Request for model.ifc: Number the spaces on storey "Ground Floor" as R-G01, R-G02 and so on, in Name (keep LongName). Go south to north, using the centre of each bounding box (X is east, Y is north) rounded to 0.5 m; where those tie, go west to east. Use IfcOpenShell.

First a look at what the model holds.

```python
import ifcopenshell
import ifcopenshell.util.element
import ifcopenshell.util.placement

model = ifcopenshell.open("model.ifc")
print(model.schema)
storey = next(s for s in model.by_type("IfcBuildingStorey") if s.Name == "Ground Floor")
spaces = [e for e in ifcopenshell.util.element.get_decomposition(storey) if e.is_a("IfcSpace")]
for e in sorted(spaces, key=lambda e: e.id()):
    origin = ifcopenshell.util.placement.get_local_placement(e.ObjectPlacement)[:3, 3]
    print(e.id(), e.Name, e.LongName, origin.round(2) + 0.0, sep=" | ")
```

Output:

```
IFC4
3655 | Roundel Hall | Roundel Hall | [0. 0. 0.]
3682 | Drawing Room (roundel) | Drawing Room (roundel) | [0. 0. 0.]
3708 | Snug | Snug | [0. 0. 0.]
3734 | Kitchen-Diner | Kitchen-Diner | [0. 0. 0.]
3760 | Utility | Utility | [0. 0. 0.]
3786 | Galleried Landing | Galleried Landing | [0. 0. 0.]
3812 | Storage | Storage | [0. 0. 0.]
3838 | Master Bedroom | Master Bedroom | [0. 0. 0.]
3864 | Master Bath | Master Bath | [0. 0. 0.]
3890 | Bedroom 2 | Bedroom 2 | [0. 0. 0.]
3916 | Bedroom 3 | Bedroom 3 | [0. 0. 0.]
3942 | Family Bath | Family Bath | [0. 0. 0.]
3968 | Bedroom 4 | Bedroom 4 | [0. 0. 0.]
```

```python
import ifcopenshell
import ifcopenshell.geom
import ifcopenshell.util.element
import ifcopenshell.util.shape

model = ifcopenshell.open("model.ifc")
settings = ifcopenshell.geom.settings()
settings.set("use-world-coords", True)


def centre(element):
    shape = ifcopenshell.geom.create_shape(settings, element)
    return ifcopenshell.util.shape.get_bbox_centroid(shape.geometry)


storey = next(s for s in model.by_type("IfcBuildingStorey") if s.Name == "Ground Floor")
spaces = [e for e in ifcopenshell.util.element.get_decomposition(storey) if e.is_a("IfcSpace")]

# Insertion points can sit at a corner or the storey origin, so sort by the geometry (in metres).
centres = {e: centre(e) for e in spaces}
spaces.sort(key=lambda e: (round(centres[e][1] / 0.5), centres[e][0]))

for i, e in enumerate(spaces, start=1):
    number = f"R-G{i:02d}"
    e.Name = number
    print(e.id(), number)

model.write("model_rev.ifc")
```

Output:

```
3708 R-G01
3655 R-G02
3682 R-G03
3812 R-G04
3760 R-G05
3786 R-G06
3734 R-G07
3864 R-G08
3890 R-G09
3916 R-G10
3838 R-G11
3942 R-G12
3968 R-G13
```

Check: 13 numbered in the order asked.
